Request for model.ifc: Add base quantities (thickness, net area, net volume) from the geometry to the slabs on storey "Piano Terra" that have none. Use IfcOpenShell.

First a look at what the model holds.

```python
import ifcopenshell
import ifcopenshell.util.element
import ifcopenshell.util.unit

model = ifcopenshell.open("model.ifc")
print(model.schema)
for unit_type in ("LENGTHUNIT", "AREAUNIT", "VOLUMEUNIT"):
    print(unit_type, ifcopenshell.util.unit.calculate_unit_scale(model, unit_type))
storey = next(s for s in model.by_type("IfcBuildingStorey") if s.Name == "Piano Terra")
slabs = [e for e in ifcopenshell.util.element.get_decomposition(storey) if e.is_a("IfcSlab")]
for e in sorted(slabs, key=lambda e: e.id()):
    print(e.id(), e.is_a(), e.Name, list(ifcopenshell.util.element.get_psets(e, qtos_only=True)), sep=" | ")
```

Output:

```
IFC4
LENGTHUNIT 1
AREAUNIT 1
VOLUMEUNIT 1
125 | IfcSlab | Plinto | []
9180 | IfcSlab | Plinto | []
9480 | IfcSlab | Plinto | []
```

```python
import ifcopenshell
import ifcopenshell.api.pset
import ifcopenshell.geom
import ifcopenshell.util.element
import ifcopenshell.util.shape
import ifcopenshell.util.unit

model = ifcopenshell.open("model.ifc")
unit_scale = ifcopenshell.util.unit.calculate_unit_scale(model)
area_scale = ifcopenshell.util.unit.calculate_unit_scale(model, "AREAUNIT")
volume_scale = ifcopenshell.util.unit.calculate_unit_scale(model, "VOLUMEUNIT")
settings = ifcopenshell.geom.settings()

storey = next(s for s in model.by_type("IfcBuildingStorey") if s.Name == "Piano Terra")
slabs = [e for e in ifcopenshell.util.element.get_decomposition(storey) if e.is_a("IfcSlab")]

for e in sorted(slabs, key=lambda e: e.id()):
    if ifcopenshell.util.element.get_psets(e, qtos_only=True, should_inherit=False):
        continue
    # Geometry comes back in metres, in the element's own axes.
    shape = ifcopenshell.geom.create_shape(settings, e)
    values = {
        "Width": ifcopenshell.util.shape.get_z(shape.geometry) / unit_scale,
        "NetArea": ifcopenshell.util.shape.get_footprint_area(shape.geometry) / area_scale,
        "NetVolume": ifcopenshell.util.shape.get_volume(shape.geometry) / volume_scale,
    }
    qto = ifcopenshell.api.pset.add_qto(model, product=e, name="Qto_SlabBaseQuantities")
    ifcopenshell.api.pset.edit_qto(model, qto=qto, properties=values)
    print(e.id(), {k: round(v, 3) for k, v in values.items()})

model.write("model_v2.ifc")
```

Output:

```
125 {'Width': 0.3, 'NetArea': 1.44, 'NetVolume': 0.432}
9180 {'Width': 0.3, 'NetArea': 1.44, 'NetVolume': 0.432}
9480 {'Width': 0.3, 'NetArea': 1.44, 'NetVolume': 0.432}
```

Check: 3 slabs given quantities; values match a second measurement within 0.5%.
